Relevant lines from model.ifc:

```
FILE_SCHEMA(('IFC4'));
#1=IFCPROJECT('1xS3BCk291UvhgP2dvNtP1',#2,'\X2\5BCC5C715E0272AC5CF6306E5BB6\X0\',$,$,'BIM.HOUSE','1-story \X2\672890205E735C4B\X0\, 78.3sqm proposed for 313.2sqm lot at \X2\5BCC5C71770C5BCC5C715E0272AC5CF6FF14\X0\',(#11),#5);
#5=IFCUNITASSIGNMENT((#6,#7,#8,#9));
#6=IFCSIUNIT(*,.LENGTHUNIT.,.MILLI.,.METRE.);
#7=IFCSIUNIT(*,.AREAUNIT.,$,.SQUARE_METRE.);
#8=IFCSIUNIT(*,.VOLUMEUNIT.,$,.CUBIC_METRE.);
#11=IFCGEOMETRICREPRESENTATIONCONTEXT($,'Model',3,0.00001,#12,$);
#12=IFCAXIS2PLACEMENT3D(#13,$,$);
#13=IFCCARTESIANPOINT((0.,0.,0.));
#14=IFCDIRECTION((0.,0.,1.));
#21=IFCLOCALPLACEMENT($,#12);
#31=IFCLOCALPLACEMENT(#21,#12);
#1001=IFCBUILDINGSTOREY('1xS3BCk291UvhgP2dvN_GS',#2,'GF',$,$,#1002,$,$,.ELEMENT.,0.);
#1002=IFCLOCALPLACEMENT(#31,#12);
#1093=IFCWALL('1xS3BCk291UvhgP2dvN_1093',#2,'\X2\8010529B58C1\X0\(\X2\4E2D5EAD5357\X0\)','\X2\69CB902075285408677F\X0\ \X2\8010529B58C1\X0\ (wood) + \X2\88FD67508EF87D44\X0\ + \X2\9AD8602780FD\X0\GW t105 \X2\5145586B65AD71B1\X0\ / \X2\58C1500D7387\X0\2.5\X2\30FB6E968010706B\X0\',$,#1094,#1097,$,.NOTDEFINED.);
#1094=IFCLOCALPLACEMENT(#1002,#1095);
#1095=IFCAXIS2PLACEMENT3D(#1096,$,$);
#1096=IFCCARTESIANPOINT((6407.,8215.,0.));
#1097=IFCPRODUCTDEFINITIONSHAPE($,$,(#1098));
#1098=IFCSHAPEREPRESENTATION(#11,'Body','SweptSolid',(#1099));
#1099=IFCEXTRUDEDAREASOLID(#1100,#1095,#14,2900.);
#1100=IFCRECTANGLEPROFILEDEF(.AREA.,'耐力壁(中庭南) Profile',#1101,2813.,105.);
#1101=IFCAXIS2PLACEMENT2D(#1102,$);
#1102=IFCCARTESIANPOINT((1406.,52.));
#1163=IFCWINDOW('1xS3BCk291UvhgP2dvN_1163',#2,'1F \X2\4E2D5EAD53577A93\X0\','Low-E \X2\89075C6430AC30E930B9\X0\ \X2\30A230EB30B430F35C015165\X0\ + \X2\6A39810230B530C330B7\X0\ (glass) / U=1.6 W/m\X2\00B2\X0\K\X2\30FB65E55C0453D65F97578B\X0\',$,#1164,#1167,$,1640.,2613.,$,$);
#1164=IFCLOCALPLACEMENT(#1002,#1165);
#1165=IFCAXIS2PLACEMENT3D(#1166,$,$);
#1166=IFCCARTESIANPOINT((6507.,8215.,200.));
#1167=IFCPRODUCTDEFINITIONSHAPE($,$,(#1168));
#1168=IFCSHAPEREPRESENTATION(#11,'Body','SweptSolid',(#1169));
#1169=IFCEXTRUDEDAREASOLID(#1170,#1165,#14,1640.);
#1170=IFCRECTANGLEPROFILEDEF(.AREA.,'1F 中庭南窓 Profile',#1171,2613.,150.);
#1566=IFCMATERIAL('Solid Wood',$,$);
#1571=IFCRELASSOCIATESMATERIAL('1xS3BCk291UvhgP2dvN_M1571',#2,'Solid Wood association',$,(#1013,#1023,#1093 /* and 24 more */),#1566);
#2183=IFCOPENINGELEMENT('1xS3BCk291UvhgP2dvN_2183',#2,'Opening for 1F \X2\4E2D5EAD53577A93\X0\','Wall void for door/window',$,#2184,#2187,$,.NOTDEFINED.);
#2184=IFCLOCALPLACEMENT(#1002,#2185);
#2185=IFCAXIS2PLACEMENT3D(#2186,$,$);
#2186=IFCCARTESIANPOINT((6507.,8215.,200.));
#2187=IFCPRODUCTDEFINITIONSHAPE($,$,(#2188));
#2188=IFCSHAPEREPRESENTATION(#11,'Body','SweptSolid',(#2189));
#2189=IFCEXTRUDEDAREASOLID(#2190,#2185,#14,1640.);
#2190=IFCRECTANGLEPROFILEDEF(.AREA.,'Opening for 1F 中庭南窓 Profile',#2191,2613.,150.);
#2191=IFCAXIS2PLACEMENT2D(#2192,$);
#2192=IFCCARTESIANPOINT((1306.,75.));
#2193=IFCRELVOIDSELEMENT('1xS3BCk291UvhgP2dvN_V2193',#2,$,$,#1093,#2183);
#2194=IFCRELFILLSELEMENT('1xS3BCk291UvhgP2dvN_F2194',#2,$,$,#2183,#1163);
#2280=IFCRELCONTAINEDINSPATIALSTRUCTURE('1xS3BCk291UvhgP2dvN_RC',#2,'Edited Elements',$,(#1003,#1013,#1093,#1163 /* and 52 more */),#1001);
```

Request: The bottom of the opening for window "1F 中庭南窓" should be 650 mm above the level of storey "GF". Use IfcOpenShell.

```python
import numpy as np
import ifcopenshell
import ifcopenshell.api.geometry
import ifcopenshell.geom
import ifcopenshell.util.element
import ifcopenshell.util.placement
import ifcopenshell.util.shape
import ifcopenshell.util.unit

model = ifcopenshell.open("model.ifc")
unit_scale = ifcopenshell.util.unit.calculate_unit_scale(model)

window = model.by_id(1163)
opening = window.FillsVoids[0].RelatingOpeningElement
storey = ifcopenshell.util.element.get_container(window, ifc_class="IfcBuildingStorey")
level = ifcopenshell.util.placement.get_local_placement(storey.ObjectPlacement)[2, 3]

# The opening's origin need not be at the sill, so measure its lowest point.
shape = ifcopenshell.geom.create_shape(ifcopenshell.geom.settings(), opening)
bottom = ifcopenshell.util.shape.get_shape_bottom_elevation(shape, shape.geometry) / unit_scale
dz = level + 0.65 / unit_scale - bottom

shift = np.array([0.0, 0.0, dz])
# The window is not placed relative to its opening, so move both.
for product in (opening, window):
    matrix = ifcopenshell.util.placement.get_local_placement(product.ObjectPlacement)
    matrix[:3, 3] += shift
    ifcopenshell.api.geometry.edit_object_placement(model, product=product, matrix=matrix, is_si=False)

print(f"moved by {dz * unit_scale:+.3f} m")

model.write("model_rev.ifc")
```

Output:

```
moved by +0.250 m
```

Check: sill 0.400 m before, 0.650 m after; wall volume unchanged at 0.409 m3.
